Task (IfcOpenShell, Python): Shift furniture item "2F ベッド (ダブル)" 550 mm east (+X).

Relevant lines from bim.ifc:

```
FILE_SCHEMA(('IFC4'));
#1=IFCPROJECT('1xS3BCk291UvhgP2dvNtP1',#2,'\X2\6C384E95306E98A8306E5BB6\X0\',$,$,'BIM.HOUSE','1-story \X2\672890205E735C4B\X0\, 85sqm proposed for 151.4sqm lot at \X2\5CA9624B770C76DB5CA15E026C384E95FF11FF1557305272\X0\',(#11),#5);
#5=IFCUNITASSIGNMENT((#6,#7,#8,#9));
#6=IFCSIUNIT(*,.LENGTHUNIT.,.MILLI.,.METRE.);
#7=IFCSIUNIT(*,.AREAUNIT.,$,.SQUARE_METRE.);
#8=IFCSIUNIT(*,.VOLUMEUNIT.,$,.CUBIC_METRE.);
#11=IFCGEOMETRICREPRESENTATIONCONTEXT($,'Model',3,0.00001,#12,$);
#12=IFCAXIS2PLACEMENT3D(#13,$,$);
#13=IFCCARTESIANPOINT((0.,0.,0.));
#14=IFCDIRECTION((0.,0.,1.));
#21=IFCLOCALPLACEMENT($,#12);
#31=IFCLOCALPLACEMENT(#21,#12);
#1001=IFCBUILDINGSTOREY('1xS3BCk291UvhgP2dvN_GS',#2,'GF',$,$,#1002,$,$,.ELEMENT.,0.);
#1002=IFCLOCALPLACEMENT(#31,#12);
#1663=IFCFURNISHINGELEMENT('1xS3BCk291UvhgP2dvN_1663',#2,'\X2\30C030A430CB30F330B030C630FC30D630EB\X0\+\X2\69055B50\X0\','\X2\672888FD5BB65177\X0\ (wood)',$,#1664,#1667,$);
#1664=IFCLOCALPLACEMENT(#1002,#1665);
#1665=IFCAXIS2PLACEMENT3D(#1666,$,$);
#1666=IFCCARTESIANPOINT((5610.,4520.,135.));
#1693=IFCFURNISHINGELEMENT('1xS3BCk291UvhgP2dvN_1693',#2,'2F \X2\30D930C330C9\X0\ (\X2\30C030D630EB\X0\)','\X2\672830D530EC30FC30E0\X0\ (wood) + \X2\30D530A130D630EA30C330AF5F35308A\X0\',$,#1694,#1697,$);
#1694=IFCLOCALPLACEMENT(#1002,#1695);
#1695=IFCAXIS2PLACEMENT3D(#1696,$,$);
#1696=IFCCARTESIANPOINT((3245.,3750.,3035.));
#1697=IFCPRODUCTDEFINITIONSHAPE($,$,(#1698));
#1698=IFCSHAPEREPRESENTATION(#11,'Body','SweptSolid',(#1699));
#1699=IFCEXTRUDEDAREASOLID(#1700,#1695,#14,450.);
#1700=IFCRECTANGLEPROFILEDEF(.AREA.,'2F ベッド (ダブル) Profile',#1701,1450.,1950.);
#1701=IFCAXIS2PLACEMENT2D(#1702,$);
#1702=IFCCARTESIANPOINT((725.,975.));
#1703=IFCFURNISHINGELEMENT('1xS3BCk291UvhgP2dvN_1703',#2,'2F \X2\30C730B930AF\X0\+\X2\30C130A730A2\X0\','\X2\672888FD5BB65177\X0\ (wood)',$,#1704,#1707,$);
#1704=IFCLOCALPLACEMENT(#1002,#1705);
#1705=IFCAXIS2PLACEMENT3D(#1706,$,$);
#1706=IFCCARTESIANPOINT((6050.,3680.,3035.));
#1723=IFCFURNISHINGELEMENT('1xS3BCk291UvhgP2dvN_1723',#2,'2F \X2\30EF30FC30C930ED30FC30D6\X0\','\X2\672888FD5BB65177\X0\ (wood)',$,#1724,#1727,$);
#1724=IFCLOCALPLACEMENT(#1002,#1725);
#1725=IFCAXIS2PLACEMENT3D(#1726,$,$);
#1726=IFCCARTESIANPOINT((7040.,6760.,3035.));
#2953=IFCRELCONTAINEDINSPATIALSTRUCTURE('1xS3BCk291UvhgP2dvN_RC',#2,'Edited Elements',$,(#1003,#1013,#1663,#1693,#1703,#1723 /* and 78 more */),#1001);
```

```python
import ifcopenshell
import ifcopenshell.api.geometry
import ifcopenshell.util.placement
import ifcopenshell.util.unit

model = ifcopenshell.open("bim.ifc")
unit_scale = ifcopenshell.util.unit.calculate_unit_scale(model)

item = model.by_id(1693)
matrix = ifcopenshell.util.placement.get_local_placement(item.ObjectPlacement)
matrix[0, 3] += 0.55 / unit_scale
ifcopenshell.api.geometry.edit_object_placement(model, product=item, matrix=matrix, is_si=False)

print(ifcopenshell.util.placement.get_local_placement(item.ObjectPlacement).round(3) + 0.0)

model.write("bim-out.ifc")
```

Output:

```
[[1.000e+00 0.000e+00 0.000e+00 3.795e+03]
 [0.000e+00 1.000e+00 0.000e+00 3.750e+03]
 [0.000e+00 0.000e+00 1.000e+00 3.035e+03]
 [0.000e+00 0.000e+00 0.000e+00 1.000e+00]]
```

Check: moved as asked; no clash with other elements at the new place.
